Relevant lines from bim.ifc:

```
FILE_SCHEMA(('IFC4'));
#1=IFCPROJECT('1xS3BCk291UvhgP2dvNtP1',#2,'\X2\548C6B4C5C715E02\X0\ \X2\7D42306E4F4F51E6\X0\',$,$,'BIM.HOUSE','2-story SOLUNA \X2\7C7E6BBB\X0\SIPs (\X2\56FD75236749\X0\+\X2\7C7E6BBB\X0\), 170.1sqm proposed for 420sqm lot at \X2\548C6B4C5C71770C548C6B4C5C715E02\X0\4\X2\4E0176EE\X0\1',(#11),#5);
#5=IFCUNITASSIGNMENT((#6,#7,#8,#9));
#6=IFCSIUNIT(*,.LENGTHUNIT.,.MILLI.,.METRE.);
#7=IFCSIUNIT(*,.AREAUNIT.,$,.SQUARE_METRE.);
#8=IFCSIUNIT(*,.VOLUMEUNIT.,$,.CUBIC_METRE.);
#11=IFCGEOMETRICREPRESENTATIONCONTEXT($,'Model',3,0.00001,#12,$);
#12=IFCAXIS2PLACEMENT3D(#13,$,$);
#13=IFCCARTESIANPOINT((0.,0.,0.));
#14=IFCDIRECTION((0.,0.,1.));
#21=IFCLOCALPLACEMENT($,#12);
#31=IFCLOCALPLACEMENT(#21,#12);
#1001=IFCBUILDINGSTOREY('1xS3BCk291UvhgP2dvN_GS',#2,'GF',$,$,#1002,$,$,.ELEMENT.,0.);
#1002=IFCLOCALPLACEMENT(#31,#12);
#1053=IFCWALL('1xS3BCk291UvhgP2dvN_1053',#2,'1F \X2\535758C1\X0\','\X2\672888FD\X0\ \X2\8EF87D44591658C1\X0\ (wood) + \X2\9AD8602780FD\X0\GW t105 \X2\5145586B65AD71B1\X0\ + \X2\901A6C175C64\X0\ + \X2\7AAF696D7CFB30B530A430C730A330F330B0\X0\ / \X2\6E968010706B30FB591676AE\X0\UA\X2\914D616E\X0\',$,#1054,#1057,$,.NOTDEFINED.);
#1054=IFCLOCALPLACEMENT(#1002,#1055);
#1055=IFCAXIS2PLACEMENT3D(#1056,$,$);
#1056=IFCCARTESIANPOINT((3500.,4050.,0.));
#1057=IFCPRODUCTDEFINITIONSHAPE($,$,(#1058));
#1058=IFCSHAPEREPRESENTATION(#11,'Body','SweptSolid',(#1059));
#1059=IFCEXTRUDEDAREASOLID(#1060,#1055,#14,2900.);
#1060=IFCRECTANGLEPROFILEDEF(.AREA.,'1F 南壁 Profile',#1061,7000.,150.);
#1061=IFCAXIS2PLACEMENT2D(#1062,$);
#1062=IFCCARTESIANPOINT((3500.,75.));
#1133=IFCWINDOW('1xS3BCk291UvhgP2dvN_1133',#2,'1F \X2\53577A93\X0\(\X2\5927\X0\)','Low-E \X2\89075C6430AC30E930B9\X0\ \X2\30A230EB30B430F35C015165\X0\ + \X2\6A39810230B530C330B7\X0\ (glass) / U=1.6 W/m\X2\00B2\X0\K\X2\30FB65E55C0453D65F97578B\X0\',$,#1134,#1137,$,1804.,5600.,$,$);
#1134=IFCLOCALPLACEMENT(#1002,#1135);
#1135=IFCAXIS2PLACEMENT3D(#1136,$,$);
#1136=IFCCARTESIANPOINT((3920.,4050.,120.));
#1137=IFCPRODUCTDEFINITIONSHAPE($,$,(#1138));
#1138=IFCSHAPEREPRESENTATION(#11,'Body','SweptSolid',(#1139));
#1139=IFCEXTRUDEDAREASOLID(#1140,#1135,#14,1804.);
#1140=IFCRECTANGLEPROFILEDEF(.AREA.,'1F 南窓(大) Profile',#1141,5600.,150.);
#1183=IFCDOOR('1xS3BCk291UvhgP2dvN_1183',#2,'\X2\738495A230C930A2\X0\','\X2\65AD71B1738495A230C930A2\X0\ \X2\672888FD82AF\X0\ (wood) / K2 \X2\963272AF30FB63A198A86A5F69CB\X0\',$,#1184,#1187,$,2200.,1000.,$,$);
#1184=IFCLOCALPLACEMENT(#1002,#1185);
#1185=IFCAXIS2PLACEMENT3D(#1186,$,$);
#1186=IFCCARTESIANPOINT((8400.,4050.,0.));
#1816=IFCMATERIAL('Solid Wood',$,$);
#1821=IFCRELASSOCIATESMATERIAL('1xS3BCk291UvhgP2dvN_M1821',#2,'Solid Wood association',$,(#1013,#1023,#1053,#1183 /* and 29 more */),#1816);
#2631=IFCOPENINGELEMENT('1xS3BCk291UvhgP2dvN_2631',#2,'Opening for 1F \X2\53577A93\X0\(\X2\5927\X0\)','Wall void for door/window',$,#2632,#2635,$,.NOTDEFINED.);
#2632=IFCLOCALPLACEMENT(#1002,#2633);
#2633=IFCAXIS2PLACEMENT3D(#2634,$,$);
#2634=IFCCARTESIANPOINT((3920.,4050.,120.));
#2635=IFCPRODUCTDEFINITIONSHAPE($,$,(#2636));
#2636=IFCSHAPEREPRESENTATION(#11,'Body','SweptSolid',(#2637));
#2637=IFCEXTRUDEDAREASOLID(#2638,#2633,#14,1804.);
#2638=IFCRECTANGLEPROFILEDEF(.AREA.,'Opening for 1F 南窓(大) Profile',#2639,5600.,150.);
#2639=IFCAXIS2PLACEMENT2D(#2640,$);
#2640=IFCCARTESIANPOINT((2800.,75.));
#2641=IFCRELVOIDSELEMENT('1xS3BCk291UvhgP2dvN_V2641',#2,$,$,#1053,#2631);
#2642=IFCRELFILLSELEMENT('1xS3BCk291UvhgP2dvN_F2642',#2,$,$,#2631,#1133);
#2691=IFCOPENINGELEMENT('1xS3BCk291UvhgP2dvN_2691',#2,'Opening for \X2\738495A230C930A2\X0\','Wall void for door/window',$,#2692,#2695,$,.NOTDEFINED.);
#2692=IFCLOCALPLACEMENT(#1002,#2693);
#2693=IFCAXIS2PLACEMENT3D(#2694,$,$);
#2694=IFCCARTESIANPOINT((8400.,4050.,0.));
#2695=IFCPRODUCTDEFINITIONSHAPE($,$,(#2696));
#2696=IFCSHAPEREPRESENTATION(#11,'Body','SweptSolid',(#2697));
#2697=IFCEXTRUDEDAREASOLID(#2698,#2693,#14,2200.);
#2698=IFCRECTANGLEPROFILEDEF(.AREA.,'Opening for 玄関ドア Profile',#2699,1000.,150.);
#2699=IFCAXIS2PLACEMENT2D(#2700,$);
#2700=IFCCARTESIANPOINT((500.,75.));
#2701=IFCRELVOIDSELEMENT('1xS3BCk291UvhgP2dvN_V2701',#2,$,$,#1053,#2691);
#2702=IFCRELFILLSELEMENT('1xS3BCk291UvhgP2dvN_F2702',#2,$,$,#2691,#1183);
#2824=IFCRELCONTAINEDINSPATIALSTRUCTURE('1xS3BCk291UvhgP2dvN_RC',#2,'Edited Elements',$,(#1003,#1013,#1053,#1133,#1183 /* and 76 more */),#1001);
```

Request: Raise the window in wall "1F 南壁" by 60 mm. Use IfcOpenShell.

```python
import numpy as np
import ifcopenshell
import ifcopenshell.api.geometry
import ifcopenshell.util.placement
import ifcopenshell.util.unit

model = ifcopenshell.open("bim.ifc")
unit_scale = ifcopenshell.util.unit.calculate_unit_scale(model)

window = model.by_guid("1xS3BCk291UvhgP2dvN_1133")
opening = window.FillsVoids[0].RelatingOpeningElement
dz = 60.0

shift = np.array([0.0, 0.0, dz])
# The window is not placed relative to its opening, so move both.
for product in (opening, window):
    matrix = ifcopenshell.util.placement.get_local_placement(product.ObjectPlacement)
    matrix[:3, 3] += shift
    ifcopenshell.api.geometry.edit_object_placement(model, product=product, matrix=matrix, is_si=False)

print(f"moved by {dz * unit_scale:+.3f} m")

model.write("bim_rev.ifc")
```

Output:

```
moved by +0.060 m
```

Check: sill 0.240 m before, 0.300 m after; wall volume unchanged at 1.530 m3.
